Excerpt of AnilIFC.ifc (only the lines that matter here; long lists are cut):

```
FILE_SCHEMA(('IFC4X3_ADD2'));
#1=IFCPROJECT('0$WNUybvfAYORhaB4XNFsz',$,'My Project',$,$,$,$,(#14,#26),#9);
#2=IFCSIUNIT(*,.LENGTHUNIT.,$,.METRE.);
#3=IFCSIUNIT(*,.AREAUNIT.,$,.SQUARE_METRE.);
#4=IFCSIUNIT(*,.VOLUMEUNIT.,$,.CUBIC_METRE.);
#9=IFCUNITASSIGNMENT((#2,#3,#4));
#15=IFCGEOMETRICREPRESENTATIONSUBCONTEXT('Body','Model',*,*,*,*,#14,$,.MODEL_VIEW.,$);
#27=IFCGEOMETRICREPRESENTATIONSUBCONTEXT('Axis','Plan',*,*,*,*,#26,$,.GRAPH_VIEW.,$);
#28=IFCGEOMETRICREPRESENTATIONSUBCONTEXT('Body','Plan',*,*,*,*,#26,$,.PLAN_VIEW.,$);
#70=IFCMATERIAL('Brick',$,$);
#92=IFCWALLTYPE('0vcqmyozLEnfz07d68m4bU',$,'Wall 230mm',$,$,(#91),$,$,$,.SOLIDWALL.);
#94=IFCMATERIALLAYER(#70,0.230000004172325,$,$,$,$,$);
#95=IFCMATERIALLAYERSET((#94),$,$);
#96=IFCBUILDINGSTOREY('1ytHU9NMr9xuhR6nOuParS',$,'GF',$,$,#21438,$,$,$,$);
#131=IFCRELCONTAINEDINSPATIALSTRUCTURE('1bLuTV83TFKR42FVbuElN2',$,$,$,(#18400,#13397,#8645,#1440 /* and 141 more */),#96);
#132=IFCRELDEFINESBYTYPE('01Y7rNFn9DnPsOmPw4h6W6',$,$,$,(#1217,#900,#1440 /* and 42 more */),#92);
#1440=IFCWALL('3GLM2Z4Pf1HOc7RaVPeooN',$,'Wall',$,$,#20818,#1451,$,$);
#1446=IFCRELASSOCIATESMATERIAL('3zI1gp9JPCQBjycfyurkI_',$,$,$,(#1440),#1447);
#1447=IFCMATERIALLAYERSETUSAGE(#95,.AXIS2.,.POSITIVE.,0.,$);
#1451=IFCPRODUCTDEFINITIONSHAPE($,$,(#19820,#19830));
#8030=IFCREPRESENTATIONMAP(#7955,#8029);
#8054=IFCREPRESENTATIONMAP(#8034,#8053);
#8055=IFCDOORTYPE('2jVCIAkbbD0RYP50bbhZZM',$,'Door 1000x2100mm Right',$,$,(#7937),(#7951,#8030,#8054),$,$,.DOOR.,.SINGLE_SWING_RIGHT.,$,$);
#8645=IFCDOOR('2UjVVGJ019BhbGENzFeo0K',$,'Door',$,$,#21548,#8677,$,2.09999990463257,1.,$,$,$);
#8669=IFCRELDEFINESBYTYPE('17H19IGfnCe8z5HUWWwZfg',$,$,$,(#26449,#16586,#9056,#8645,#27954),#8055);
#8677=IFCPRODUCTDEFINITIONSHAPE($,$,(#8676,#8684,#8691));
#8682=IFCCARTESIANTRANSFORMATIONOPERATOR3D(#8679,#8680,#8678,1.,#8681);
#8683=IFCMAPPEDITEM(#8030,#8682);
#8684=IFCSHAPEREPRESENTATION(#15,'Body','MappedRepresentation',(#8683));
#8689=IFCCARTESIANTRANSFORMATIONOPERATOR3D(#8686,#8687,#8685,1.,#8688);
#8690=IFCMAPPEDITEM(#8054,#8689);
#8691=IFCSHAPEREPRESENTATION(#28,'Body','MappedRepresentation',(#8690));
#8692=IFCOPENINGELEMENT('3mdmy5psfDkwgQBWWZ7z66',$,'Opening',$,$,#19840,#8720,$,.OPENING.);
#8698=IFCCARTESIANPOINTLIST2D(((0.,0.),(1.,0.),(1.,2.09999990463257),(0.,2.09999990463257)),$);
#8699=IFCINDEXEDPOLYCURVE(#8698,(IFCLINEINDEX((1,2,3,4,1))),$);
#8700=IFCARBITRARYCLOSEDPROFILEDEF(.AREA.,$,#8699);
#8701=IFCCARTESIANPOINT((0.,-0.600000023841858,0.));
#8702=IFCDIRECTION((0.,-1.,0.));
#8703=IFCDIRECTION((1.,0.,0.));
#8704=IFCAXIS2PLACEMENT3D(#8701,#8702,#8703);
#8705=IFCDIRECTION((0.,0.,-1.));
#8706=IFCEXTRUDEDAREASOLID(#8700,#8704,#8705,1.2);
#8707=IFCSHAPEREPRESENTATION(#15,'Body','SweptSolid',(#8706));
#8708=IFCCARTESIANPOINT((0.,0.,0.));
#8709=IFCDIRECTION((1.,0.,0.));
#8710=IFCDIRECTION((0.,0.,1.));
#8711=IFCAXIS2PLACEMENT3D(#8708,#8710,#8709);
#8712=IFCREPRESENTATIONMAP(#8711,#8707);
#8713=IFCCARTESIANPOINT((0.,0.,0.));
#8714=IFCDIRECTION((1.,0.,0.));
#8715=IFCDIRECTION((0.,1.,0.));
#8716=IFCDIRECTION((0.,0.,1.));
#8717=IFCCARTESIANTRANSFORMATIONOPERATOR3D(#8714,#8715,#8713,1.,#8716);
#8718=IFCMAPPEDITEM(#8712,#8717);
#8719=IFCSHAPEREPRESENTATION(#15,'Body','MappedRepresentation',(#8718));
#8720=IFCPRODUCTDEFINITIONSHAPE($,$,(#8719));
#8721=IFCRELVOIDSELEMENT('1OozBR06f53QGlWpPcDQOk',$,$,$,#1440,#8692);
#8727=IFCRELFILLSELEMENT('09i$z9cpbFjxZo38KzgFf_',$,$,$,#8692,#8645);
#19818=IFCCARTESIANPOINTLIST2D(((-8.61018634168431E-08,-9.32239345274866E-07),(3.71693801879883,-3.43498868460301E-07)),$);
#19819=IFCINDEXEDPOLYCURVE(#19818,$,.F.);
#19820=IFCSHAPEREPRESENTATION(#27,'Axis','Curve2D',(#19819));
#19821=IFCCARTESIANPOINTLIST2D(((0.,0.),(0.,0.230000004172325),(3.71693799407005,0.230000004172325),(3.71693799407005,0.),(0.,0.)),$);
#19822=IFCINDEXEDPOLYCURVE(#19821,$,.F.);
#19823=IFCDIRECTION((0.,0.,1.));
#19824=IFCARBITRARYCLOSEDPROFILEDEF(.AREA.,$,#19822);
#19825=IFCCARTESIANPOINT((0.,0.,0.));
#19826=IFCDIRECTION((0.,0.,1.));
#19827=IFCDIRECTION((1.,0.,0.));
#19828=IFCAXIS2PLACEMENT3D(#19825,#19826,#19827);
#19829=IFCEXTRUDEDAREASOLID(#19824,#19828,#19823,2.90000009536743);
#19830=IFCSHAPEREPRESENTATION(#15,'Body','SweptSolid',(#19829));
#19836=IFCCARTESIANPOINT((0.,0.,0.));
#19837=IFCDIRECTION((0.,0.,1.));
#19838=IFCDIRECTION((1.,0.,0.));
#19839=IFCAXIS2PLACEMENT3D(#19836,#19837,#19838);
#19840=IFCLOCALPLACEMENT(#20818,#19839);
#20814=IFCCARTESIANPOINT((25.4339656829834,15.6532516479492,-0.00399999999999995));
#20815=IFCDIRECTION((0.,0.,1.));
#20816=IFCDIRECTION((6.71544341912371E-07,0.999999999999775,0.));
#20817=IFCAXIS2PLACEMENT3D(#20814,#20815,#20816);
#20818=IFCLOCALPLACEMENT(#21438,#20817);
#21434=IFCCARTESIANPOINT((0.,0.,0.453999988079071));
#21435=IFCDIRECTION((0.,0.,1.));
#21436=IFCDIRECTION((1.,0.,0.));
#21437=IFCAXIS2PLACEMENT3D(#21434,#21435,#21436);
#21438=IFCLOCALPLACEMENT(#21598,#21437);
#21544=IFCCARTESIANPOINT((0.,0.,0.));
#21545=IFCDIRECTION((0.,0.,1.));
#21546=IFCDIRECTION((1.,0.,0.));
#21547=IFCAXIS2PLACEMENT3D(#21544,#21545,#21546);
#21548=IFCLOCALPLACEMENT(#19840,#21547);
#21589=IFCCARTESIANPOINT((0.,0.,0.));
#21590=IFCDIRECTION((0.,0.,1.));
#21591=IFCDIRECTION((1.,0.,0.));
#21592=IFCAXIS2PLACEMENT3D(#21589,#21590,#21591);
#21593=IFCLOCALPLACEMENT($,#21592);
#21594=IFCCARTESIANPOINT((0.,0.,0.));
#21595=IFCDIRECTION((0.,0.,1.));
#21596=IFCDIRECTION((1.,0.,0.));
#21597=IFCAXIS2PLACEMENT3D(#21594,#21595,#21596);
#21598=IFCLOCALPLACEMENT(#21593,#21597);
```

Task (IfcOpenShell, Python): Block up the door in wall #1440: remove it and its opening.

```python
import ifcopenshell
import ifcopenshell.api.feature
import ifcopenshell.api.root
import ifcopenshell.geom
import ifcopenshell.util.shape

model = ifcopenshell.open("AnilIFC.ifc")
settings = ifcopenshell.geom.settings()


def volume(element):
    """Net volume in cubic metres, openings subtracted."""
    shape = ifcopenshell.geom.create_shape(settings, element)
    return ifcopenshell.util.shape.get_volume(shape.geometry)


door = model.by_guid("2UjVVGJ019BhbGENzFeo0K")
opening = door.FillsVoids[0].RelatingOpeningElement
wall = opening.VoidsElements[0].RelatingBuildingElement
before = volume(wall)

ifcopenshell.api.root.remove_product(model, product=door)
ifcopenshell.api.feature.remove_feature(model, feature=opening)

after = volume(wall)

print(f"wall volume {before:.3f} -> {after:.3f} m3")

model.write("AnilIFC-out.ifc")
```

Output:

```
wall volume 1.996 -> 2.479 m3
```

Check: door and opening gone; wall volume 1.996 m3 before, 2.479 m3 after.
